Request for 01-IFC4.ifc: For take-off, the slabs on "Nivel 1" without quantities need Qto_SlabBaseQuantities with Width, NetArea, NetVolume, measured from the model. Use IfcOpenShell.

First a look at what the model holds.

```python
import ifcopenshell
import ifcopenshell.util.element
import ifcopenshell.util.unit

model = ifcopenshell.open("01-IFC4.ifc")
print(model.schema)
for unit_type in ("LENGTHUNIT", "AREAUNIT", "VOLUMEUNIT"):
    print(unit_type, ifcopenshell.util.unit.calculate_unit_scale(model, unit_type))
storey = next(s for s in model.by_type("IfcBuildingStorey") if s.Name == "Nivel 1")
slabs = [e for e in ifcopenshell.util.element.get_decomposition(storey) if e.is_a("IfcSlab")]
for e in sorted(slabs, key=lambda e: e.id()):
    print(e.id(), e.is_a(), e.Name, list(ifcopenshell.util.element.get_psets(e, qtos_only=True)), sep=" | ")
```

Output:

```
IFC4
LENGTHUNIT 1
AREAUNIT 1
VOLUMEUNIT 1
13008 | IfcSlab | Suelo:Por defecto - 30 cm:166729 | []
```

```python
import ifcopenshell
import ifcopenshell.api.pset
import ifcopenshell.geom
import ifcopenshell.util.element
import ifcopenshell.util.shape
import ifcopenshell.util.unit

model = ifcopenshell.open("01-IFC4.ifc")
unit_scale = ifcopenshell.util.unit.calculate_unit_scale(model)
area_scale = ifcopenshell.util.unit.calculate_unit_scale(model, "AREAUNIT")
volume_scale = ifcopenshell.util.unit.calculate_unit_scale(model, "VOLUMEUNIT")
settings = ifcopenshell.geom.settings()

storey = next(s for s in model.by_type("IfcBuildingStorey") if s.Name == "Nivel 1")
slabs = [e for e in ifcopenshell.util.element.get_decomposition(storey) if e.is_a("IfcSlab")]

for e in sorted(slabs, key=lambda e: e.id()):
    if ifcopenshell.util.element.get_psets(e, qtos_only=True, should_inherit=False):
        continue
    # Geometry comes back in metres, in the element's own axes.
    shape = ifcopenshell.geom.create_shape(settings, e)
    values = {
        "Width": ifcopenshell.util.shape.get_z(shape.geometry) / unit_scale,
        "NetArea": ifcopenshell.util.shape.get_footprint_area(shape.geometry) / area_scale,
        "NetVolume": ifcopenshell.util.shape.get_volume(shape.geometry) / volume_scale,
    }
    qto = ifcopenshell.api.pset.add_qto(model, product=e, name="Qto_SlabBaseQuantities")
    ifcopenshell.api.pset.edit_qto(model, qto=qto, properties=values)
    print(e.id(), {k: round(v, 3) for k, v in values.items()})

model.write("01-IFC4_v2.ifc")
```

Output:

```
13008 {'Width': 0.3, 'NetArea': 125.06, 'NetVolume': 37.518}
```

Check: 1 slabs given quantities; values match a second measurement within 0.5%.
